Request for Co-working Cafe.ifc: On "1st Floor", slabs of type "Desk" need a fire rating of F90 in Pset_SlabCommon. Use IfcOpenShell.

First a look at what the model holds.

```python
import ifcopenshell
import ifcopenshell.util.element

model = ifcopenshell.open("Co-working Cafe.ifc")
print(model.schema)
storey = next(s for s in model.by_type("IfcBuildingStorey") if s.Name == "1st Floor")
slabs = [e for e in ifcopenshell.util.element.get_decomposition(storey) if e.is_a("IfcSlab")]
seen = {}
for e in slabs:
    element_type = ifcopenshell.util.element.get_type(e)
    key = (element_type.Name if element_type != e and element_type else None, ifcopenshell.util.element.get_pset(e, "Pset_SlabCommon", "FireRating"))
    seen[key] = seen.get(key, 0) + 1
for (name, value), count in sorted(seen.items(), key=str):
    print(count, "x", name, "|", value)
```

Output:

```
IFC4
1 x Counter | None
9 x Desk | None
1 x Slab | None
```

```python
import ifcopenshell
import ifcopenshell.api.pset
import ifcopenshell.util.element

model = ifcopenshell.open("Co-working Cafe.ifc")

storey = next(s for s in model.by_type("IfcBuildingStorey") if s.Name == "1st Floor")
slabs = [e for e in ifcopenshell.util.element.get_decomposition(storey) if e.is_a("IfcSlab")]

count = 0
for e in slabs:
    element_type = ifcopenshell.util.element.get_type(e)
    if element_type in (None, e) or element_type.Name != "Desk":
        continue
    # add_pset returns the element's existing set when there is one.
    pset = ifcopenshell.api.pset.add_pset(model, product=e, name="Pset_SlabCommon")
    ifcopenshell.api.pset.edit_pset(model, pset=pset, properties={"FireRating": "F90"})
    count += 1

print(count, "slabs updated")

model.write("Co-working Cafe_updated.ifc")
```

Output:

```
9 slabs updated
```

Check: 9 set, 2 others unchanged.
